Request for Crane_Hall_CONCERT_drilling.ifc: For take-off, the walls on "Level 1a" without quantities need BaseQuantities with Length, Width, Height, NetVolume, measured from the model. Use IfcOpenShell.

First a look at what the model holds.

```python
import ifcopenshell
import ifcopenshell.util.element
import ifcopenshell.util.unit

model = ifcopenshell.open("Crane_Hall_CONCERT_drilling.ifc")
print(model.schema)
for unit_type in ("LENGTHUNIT", "AREAUNIT", "VOLUMEUNIT"):
    print(unit_type, ifcopenshell.util.unit.calculate_unit_scale(model, unit_type))
storey = next(s for s in model.by_type("IfcBuildingStorey") if s.Name == "Level 1a")
walls = [e for e in ifcopenshell.util.element.get_decomposition(storey) if e.is_a("IfcWall")]
for e in sorted(walls, key=lambda e: e.id()):
    print(e.id(), e.is_a(), e.Name, list(ifcopenshell.util.element.get_psets(e, qtos_only=True)), sep=" | ")
```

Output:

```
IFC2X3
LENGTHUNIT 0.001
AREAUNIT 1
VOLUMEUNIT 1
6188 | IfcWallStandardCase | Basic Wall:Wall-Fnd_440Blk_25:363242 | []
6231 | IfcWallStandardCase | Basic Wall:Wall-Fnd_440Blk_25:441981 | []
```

```python
import ifcopenshell
import ifcopenshell.api.pset
import ifcopenshell.geom
import ifcopenshell.util.element
import ifcopenshell.util.shape
import ifcopenshell.util.unit

model = ifcopenshell.open("Crane_Hall_CONCERT_drilling.ifc")
unit_scale = ifcopenshell.util.unit.calculate_unit_scale(model)
volume_scale = ifcopenshell.util.unit.calculate_unit_scale(model, "VOLUMEUNIT")
settings = ifcopenshell.geom.settings()

storey = next(s for s in model.by_type("IfcBuildingStorey") if s.Name == "Level 1a")
walls = [e for e in ifcopenshell.util.element.get_decomposition(storey) if e.is_a("IfcWall")]

for e in sorted(walls, key=lambda e: e.id()):
    if ifcopenshell.util.element.get_psets(e, qtos_only=True, should_inherit=False):
        continue
    # Geometry comes back in metres, in the element's own axes.
    shape = ifcopenshell.geom.create_shape(settings, e)
    values = {
        "Length": ifcopenshell.util.shape.get_x(shape.geometry) / unit_scale,
        "Width": ifcopenshell.util.shape.get_y(shape.geometry) / unit_scale,
        "Height": ifcopenshell.util.shape.get_z(shape.geometry) / unit_scale,
        "NetVolume": ifcopenshell.util.shape.get_volume(shape.geometry) / volume_scale,
    }
    qto = ifcopenshell.api.pset.add_qto(model, product=e, name="BaseQuantities")
    ifcopenshell.api.pset.edit_qto(model, qto=qto, properties=values)
    print(e.id(), {k: round(v, 3) for k, v in values.items()})

model.write("Crane_Hall_CONCERT_drilling_rev.ifc")
```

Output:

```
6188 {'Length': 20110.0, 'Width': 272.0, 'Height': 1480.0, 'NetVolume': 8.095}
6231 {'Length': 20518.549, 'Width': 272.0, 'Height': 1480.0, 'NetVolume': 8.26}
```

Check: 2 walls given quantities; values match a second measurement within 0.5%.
